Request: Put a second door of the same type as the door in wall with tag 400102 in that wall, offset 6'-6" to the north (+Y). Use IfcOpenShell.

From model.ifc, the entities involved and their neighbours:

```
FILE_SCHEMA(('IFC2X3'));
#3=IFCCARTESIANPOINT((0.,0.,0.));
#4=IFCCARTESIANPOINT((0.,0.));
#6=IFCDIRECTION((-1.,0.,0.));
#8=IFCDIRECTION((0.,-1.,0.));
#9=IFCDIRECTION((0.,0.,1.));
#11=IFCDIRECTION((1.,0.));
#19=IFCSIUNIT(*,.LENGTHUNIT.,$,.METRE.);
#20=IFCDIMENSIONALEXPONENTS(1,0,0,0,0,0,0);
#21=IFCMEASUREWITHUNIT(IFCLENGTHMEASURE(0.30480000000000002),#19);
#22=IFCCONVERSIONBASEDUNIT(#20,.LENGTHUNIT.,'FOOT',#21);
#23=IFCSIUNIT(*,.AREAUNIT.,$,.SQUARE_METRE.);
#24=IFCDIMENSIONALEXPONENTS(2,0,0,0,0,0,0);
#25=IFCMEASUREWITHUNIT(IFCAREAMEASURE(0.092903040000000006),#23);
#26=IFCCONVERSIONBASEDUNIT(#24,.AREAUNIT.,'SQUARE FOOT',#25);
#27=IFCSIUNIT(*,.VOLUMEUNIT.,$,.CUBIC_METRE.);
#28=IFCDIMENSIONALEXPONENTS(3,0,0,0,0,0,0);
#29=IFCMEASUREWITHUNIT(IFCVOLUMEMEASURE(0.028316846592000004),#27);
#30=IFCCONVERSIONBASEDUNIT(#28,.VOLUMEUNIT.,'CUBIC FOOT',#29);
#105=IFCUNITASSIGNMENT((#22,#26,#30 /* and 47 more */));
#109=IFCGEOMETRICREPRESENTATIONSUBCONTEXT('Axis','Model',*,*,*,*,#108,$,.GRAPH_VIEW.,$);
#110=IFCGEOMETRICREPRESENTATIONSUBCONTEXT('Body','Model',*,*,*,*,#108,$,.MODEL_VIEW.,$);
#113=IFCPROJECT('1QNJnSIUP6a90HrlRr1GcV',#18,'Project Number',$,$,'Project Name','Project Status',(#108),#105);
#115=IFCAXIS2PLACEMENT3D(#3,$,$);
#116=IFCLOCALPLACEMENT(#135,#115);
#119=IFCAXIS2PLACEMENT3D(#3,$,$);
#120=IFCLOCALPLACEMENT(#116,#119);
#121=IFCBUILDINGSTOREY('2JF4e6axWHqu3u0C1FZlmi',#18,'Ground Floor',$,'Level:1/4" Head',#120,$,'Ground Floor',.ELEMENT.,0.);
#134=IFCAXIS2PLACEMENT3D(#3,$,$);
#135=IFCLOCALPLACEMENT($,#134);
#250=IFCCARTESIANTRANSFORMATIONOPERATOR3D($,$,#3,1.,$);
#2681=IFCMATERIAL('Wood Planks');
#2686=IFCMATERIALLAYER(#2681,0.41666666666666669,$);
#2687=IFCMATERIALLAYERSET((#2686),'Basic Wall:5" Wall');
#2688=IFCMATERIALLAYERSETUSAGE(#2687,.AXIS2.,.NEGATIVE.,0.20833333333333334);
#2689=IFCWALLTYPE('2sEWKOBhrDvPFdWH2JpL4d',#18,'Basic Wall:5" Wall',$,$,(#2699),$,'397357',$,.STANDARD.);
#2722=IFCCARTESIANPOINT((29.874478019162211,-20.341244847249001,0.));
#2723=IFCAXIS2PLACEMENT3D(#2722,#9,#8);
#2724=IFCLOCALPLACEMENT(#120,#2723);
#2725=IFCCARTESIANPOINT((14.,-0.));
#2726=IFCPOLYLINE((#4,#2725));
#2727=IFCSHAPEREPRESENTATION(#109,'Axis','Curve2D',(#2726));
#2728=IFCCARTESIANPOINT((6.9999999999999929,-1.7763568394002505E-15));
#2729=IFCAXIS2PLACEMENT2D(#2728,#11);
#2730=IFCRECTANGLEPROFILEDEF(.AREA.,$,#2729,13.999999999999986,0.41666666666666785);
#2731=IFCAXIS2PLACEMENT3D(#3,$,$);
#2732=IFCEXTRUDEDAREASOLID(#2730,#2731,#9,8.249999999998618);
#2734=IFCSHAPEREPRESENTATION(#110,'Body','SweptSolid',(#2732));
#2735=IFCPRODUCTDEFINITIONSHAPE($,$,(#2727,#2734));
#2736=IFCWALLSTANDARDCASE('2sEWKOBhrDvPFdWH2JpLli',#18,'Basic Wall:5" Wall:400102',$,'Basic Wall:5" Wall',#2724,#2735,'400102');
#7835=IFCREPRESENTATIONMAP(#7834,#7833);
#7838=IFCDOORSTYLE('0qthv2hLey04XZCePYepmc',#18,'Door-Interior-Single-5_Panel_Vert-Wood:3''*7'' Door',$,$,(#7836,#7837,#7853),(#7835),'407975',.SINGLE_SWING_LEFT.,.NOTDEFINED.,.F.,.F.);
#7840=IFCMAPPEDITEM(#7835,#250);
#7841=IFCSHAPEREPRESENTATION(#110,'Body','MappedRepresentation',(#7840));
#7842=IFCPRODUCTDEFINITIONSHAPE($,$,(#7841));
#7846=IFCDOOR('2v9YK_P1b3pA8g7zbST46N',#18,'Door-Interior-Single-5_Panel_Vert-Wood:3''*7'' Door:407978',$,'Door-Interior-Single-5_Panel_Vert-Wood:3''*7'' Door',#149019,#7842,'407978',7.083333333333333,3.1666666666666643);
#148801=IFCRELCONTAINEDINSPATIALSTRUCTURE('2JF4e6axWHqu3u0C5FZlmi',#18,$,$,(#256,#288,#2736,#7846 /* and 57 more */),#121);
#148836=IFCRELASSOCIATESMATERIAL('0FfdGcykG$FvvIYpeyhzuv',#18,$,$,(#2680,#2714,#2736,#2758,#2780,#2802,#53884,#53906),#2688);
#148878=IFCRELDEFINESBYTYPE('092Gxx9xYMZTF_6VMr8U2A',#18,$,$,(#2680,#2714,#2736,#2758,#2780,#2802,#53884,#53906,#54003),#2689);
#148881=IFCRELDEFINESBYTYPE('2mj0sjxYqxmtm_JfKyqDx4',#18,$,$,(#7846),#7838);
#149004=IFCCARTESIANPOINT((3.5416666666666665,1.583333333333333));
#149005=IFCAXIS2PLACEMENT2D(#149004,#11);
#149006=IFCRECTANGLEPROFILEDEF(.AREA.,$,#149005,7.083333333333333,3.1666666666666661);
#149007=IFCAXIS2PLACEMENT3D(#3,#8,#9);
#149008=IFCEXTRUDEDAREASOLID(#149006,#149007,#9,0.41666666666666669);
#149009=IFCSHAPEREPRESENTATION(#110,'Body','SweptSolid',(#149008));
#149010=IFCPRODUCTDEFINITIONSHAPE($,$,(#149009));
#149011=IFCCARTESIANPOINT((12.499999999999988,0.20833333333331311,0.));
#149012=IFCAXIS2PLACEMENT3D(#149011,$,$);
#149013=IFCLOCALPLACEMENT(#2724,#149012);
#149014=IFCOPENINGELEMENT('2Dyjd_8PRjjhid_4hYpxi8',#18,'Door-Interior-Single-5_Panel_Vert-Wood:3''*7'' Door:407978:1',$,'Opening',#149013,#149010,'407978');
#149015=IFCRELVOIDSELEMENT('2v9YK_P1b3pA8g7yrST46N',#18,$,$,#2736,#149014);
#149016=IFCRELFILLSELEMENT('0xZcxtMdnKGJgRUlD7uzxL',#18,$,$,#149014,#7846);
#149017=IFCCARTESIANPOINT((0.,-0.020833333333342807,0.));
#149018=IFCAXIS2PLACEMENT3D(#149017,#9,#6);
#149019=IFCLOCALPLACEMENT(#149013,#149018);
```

```python
import ifcopenshell
import ifcopenshell.api.feature
import ifcopenshell.api.geometry
import ifcopenshell.api.root
import ifcopenshell.geom
import ifcopenshell.util.element
import ifcopenshell.util.placement
import ifcopenshell.util.shape
import ifcopenshell.util.unit

model = ifcopenshell.open("model.ifc")
unit_scale = ifcopenshell.util.unit.calculate_unit_scale(model)
settings = ifcopenshell.geom.settings()


def volume(element):
    """Net volume in cubic metres, openings subtracted."""
    shape = ifcopenshell.geom.create_shape(settings, element)
    return ifcopenshell.util.shape.get_volume(shape.geometry)


def reuse_history(source, copy):
    """copy_class also copies each property set's owner history, people and application; keep the originals."""
    for rel in copy.IsDefinedBy:
        if rel.is_a("IfcRelDefinesByProperties") and (history := rel.RelatingPropertyDefinition.OwnerHistory):
            rel.RelatingPropertyDefinition.OwnerHistory = source.OwnerHistory
            ifcopenshell.util.element.remove_deep2(model, history)


door = model.by_guid("2v9YK_P1b3pA8g7zbST46N")
opening = door.FillsVoids[0].RelatingOpeningElement
wall = opening.VoidsElements[0].RelatingBuildingElement
before = volume(wall)
shift = ifcopenshell.util.placement.get_local_placement(wall.ObjectPlacement)[:3, 0] * -78 * 0.0254 / unit_scale

# copy_class copies the void relationship, type, container and properties, but no geometry.
new_opening = ifcopenshell.api.root.copy_class(model, product=opening)
new_opening.Representation = ifcopenshell.util.element.copy_deep(
    model, opening.Representation, exclude=["IfcGeometricRepresentationContext", "IfcRepresentationMap"]
)
new_opening.Name = "Door-Interior-Single-5_Panel_Vert-Wood:3'*7' Door"
new_opening.Tag = None
new_door = ifcopenshell.api.root.copy_class(model, product=door)
new_door.Representation = ifcopenshell.util.element.copy_deep(
    model, door.Representation, exclude=["IfcGeometricRepresentationContext", "IfcRepresentationMap"]
)
new_door.Name = "Door-Interior-Single-5_Panel_Vert-Wood:3'*7' Door"
new_door.Tag = None
reuse_history(door, new_door)
fills = ifcopenshell.api.feature.add_filling(model, opening=new_opening, element=new_door)
fills.OwnerHistory = new_door.OwnerHistory  # required in IFC2X3

for old, new in ((opening, new_opening), (door, new_door)):
    matrix = ifcopenshell.util.placement.get_local_placement(old.ObjectPlacement)
    matrix[:3, 3] += shift
    ifcopenshell.api.geometry.edit_object_placement(model, product=new, matrix=matrix, is_si=False)

after = volume(wall)

print(f"wall volume {before:.3f} -> {after:.3f} m3")

model.write("model-out.ifc")
```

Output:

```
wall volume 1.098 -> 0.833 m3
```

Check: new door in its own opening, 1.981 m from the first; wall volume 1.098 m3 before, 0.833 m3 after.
